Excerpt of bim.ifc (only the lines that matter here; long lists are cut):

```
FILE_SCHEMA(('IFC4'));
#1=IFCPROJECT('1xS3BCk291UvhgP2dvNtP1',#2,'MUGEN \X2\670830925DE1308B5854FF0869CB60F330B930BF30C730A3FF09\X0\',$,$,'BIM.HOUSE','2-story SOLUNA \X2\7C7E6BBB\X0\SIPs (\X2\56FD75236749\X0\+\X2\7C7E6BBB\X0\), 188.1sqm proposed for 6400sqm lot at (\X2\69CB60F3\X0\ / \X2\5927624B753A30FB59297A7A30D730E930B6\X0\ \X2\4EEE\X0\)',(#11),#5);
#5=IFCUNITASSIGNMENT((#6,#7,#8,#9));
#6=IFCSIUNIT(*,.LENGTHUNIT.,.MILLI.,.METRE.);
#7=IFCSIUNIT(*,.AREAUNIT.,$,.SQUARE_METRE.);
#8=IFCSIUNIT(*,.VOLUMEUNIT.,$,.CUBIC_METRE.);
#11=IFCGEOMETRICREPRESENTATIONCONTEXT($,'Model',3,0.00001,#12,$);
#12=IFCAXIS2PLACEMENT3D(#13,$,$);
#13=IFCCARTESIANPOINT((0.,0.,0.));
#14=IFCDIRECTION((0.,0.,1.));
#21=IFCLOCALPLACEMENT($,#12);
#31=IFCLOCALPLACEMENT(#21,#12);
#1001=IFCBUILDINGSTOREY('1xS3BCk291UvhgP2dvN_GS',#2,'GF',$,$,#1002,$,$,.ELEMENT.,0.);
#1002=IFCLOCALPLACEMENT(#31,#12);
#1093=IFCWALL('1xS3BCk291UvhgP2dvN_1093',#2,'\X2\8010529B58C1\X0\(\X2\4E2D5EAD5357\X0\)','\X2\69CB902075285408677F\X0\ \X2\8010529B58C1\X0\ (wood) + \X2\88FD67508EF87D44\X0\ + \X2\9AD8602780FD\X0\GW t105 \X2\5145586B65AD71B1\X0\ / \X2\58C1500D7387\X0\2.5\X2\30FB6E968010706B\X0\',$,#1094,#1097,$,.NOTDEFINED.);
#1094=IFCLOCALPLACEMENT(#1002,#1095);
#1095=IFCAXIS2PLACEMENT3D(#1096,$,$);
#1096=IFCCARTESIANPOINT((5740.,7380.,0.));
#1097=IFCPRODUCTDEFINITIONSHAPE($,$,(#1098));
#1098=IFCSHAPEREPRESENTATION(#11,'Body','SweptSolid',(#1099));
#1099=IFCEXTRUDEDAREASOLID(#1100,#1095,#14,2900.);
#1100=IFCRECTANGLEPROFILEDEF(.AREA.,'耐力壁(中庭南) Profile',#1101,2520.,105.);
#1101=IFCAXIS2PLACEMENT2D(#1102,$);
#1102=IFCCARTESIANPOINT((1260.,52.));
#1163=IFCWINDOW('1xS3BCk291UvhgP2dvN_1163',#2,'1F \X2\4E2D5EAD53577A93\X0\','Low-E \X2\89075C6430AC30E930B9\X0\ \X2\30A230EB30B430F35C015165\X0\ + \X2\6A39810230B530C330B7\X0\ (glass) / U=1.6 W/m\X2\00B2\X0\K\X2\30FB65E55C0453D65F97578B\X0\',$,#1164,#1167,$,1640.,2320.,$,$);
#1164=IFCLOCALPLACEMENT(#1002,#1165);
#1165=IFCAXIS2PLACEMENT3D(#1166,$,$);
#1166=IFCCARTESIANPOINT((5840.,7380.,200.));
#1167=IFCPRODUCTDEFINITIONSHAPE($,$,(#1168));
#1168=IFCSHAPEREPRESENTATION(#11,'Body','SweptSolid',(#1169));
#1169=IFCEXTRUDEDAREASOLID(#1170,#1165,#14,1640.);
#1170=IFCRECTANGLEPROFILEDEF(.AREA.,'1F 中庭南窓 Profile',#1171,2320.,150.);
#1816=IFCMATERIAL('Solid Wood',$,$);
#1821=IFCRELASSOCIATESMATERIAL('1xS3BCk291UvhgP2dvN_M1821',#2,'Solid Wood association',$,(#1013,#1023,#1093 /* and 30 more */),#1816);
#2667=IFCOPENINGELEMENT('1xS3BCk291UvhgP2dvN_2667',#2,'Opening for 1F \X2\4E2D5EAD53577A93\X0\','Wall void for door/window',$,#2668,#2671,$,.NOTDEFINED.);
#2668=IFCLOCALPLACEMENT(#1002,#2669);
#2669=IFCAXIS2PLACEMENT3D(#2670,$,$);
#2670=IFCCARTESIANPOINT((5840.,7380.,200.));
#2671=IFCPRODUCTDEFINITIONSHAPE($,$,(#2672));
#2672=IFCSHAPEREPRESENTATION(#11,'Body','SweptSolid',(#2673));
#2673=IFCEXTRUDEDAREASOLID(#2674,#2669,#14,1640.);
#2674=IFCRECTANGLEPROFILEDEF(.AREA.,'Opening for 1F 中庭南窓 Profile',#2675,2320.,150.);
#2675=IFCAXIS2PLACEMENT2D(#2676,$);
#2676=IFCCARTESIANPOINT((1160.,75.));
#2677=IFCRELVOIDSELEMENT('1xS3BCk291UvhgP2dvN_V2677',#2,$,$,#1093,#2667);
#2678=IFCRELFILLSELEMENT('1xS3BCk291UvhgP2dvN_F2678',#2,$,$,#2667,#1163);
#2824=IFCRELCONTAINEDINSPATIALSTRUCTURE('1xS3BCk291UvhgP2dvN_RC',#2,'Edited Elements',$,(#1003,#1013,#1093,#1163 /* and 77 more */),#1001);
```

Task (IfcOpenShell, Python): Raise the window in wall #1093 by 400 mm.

```python
import numpy as np
import ifcopenshell
import ifcopenshell.api.geometry
import ifcopenshell.util.placement
import ifcopenshell.util.unit

model = ifcopenshell.open("bim.ifc")
unit_scale = ifcopenshell.util.unit.calculate_unit_scale(model)

window = model.by_guid("1xS3BCk291UvhgP2dvN_1163")
opening = window.FillsVoids[0].RelatingOpeningElement
dz = 400.0

shift = np.array([0.0, 0.0, dz])
# The window is not placed relative to its opening, so move both.
for product in (opening, window):
    matrix = ifcopenshell.util.placement.get_local_placement(product.ObjectPlacement)
    matrix[:3, 3] += shift
    ifcopenshell.api.geometry.edit_object_placement(model, product=product, matrix=matrix, is_si=False)

print(f"moved by {dz * unit_scale:+.3f} m")

model.write("bim_v2.ifc")
```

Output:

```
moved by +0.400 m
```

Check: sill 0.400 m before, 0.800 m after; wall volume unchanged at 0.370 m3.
